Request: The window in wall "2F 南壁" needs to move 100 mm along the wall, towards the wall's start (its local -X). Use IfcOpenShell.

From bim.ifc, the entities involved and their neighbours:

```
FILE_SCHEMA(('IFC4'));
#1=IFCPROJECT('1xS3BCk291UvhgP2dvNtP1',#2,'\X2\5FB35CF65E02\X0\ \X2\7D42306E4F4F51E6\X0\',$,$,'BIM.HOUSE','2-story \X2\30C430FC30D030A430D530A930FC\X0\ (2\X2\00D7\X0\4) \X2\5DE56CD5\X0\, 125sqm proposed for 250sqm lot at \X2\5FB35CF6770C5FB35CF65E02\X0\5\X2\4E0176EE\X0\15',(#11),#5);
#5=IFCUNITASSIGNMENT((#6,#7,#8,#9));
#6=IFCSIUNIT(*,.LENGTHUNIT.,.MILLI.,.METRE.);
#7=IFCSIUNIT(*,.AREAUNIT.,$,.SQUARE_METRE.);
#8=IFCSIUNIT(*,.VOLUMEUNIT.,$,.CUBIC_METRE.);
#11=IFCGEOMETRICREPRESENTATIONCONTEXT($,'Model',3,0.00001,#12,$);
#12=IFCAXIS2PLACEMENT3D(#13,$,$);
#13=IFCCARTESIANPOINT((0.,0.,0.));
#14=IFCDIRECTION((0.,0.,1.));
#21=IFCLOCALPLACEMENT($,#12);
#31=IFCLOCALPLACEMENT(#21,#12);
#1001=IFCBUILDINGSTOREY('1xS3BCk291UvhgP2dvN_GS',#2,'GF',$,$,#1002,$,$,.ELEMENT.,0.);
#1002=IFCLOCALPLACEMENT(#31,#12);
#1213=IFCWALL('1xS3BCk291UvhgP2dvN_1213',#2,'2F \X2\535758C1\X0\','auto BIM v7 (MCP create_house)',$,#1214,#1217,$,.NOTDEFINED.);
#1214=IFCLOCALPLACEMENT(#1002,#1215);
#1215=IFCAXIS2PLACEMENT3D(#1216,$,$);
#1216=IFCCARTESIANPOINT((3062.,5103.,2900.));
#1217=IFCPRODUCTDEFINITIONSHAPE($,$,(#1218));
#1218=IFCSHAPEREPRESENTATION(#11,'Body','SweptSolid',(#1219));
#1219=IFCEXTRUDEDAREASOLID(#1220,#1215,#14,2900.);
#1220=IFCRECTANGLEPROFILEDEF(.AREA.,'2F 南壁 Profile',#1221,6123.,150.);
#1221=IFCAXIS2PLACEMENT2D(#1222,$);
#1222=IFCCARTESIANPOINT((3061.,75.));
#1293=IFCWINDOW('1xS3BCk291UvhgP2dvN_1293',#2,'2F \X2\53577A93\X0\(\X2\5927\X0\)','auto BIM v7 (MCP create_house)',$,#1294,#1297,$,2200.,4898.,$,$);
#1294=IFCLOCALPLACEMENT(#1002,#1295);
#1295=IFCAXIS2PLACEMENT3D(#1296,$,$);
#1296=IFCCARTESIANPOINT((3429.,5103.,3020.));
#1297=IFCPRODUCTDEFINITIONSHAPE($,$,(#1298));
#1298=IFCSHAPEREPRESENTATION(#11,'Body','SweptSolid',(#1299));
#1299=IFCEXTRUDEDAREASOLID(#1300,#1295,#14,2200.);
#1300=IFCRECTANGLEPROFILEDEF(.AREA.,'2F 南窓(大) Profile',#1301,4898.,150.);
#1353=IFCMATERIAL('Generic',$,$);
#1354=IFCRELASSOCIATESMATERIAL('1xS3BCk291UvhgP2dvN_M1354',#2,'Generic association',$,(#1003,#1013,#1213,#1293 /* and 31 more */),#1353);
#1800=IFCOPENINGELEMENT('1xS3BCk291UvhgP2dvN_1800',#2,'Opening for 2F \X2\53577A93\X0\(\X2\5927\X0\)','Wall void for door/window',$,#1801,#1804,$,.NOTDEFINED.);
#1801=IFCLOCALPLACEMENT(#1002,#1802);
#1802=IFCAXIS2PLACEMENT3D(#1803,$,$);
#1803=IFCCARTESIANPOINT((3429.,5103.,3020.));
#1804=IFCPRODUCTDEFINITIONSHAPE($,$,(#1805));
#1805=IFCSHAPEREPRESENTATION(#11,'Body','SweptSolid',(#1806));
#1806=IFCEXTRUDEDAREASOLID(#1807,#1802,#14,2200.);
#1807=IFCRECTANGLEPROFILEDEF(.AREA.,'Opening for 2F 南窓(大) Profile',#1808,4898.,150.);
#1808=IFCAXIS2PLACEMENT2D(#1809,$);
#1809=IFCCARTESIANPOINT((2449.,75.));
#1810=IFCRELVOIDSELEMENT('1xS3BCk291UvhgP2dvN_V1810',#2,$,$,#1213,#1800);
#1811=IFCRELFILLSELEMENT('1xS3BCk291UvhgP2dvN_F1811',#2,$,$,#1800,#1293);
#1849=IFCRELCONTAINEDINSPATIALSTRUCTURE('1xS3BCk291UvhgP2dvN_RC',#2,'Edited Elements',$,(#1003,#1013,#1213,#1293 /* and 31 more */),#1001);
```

```python
import ifcopenshell
import ifcopenshell.api.geometry
import ifcopenshell.util.placement
import ifcopenshell.util.unit

model = ifcopenshell.open("bim.ifc")
unit_scale = ifcopenshell.util.unit.calculate_unit_scale(model)

window = model.by_id(1293)
opening = window.FillsVoids[0].RelatingOpeningElement
wall = opening.VoidsElements[0].RelatingBuildingElement

wall_matrix = ifcopenshell.util.placement.get_local_placement(wall.ObjectPlacement)
shift = wall_matrix[:3, 0] * -0.1 / unit_scale
before = ifcopenshell.util.placement.get_local_placement(window.ObjectPlacement)[:3, 3].copy()

# The window is not placed relative to its opening, so move both.
for product in (opening, window):
    matrix = ifcopenshell.util.placement.get_local_placement(product.ObjectPlacement)
    matrix[:3, 3] += shift
    ifcopenshell.api.geometry.edit_object_placement(model, product=product, matrix=matrix, is_si=False)

after = ifcopenshell.util.placement.get_local_placement(window.ObjectPlacement)[:3, 3]
print("window moved by", (after - before).round(3) + 0.0)

model.write("bim_rev.ifc")
```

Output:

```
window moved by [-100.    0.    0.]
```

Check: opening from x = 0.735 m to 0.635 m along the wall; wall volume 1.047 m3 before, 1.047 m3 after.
